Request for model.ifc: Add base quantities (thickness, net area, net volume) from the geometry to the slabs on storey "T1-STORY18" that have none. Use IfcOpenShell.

First a look at what the model holds.

```python
import ifcopenshell
import ifcopenshell.util.element
import ifcopenshell.util.unit

model = ifcopenshell.open("model.ifc")
print(model.schema)
for unit_type in ("LENGTHUNIT", "AREAUNIT", "VOLUMEUNIT"):
    print(unit_type, ifcopenshell.util.unit.calculate_unit_scale(model, unit_type))
storey = next(s for s in model.by_type("IfcBuildingStorey") if s.Name == "T1-STORY18")
slabs = [e for e in ifcopenshell.util.element.get_decomposition(storey) if e.is_a("IfcSlab")]
for e in sorted(slabs, key=lambda e: e.id()):
    print(e.id(), e.is_a(), e.Name, list(ifcopenshell.util.element.get_psets(e, qtos_only=True)), sep=" | ")
```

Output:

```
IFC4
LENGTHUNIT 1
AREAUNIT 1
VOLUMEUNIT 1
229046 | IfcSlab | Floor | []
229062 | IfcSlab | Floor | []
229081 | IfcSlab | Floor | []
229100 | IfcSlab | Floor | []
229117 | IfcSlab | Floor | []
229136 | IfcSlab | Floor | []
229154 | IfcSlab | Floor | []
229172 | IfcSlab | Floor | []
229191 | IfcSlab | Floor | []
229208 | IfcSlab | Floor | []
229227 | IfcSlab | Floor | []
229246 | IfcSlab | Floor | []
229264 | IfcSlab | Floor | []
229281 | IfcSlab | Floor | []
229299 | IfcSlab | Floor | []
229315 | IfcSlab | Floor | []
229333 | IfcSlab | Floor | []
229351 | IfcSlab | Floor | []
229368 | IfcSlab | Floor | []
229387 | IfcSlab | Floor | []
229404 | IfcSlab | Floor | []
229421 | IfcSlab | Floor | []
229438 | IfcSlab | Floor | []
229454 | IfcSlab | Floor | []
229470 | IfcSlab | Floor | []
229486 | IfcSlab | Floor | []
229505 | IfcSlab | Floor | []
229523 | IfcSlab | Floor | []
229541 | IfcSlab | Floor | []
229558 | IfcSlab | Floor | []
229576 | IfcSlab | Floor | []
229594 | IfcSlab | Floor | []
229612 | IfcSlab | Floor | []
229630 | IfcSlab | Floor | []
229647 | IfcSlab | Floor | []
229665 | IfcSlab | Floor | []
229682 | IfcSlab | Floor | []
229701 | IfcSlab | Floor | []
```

```python
import ifcopenshell
import ifcopenshell.api.pset
import ifcopenshell.geom
import ifcopenshell.util.element
import ifcopenshell.util.shape
import ifcopenshell.util.unit

model = ifcopenshell.open("model.ifc")
unit_scale = ifcopenshell.util.unit.calculate_unit_scale(model)
area_scale = ifcopenshell.util.unit.calculate_unit_scale(model, "AREAUNIT")
volume_scale = ifcopenshell.util.unit.calculate_unit_scale(model, "VOLUMEUNIT")
settings = ifcopenshell.geom.settings()

storey = next(s for s in model.by_type("IfcBuildingStorey") if s.Name == "T1-STORY18")
slabs = [e for e in ifcopenshell.util.element.get_decomposition(storey) if e.is_a("IfcSlab")]

for e in sorted(slabs, key=lambda e: e.id()):
    if ifcopenshell.util.element.get_psets(e, qtos_only=True, should_inherit=False):
        continue
    # Geometry comes back in metres, in the element's own axes.
    shape = ifcopenshell.geom.create_shape(settings, e)
    values = {
        "Width": ifcopenshell.util.shape.get_z(shape.geometry) / unit_scale,
        "NetArea": ifcopenshell.util.shape.get_footprint_area(shape.geometry) / area_scale,
        "NetVolume": ifcopenshell.util.shape.get_volume(shape.geometry) / volume_scale,
    }
    qto = ifcopenshell.api.pset.add_qto(model, product=e, name="Qto_SlabBaseQuantities")
    ifcopenshell.api.pset.edit_qto(model, qto=qto, properties=values)
    print(e.id(), {k: round(v, 3) for k, v in values.items()})

model.write("model_updated.ifc")
```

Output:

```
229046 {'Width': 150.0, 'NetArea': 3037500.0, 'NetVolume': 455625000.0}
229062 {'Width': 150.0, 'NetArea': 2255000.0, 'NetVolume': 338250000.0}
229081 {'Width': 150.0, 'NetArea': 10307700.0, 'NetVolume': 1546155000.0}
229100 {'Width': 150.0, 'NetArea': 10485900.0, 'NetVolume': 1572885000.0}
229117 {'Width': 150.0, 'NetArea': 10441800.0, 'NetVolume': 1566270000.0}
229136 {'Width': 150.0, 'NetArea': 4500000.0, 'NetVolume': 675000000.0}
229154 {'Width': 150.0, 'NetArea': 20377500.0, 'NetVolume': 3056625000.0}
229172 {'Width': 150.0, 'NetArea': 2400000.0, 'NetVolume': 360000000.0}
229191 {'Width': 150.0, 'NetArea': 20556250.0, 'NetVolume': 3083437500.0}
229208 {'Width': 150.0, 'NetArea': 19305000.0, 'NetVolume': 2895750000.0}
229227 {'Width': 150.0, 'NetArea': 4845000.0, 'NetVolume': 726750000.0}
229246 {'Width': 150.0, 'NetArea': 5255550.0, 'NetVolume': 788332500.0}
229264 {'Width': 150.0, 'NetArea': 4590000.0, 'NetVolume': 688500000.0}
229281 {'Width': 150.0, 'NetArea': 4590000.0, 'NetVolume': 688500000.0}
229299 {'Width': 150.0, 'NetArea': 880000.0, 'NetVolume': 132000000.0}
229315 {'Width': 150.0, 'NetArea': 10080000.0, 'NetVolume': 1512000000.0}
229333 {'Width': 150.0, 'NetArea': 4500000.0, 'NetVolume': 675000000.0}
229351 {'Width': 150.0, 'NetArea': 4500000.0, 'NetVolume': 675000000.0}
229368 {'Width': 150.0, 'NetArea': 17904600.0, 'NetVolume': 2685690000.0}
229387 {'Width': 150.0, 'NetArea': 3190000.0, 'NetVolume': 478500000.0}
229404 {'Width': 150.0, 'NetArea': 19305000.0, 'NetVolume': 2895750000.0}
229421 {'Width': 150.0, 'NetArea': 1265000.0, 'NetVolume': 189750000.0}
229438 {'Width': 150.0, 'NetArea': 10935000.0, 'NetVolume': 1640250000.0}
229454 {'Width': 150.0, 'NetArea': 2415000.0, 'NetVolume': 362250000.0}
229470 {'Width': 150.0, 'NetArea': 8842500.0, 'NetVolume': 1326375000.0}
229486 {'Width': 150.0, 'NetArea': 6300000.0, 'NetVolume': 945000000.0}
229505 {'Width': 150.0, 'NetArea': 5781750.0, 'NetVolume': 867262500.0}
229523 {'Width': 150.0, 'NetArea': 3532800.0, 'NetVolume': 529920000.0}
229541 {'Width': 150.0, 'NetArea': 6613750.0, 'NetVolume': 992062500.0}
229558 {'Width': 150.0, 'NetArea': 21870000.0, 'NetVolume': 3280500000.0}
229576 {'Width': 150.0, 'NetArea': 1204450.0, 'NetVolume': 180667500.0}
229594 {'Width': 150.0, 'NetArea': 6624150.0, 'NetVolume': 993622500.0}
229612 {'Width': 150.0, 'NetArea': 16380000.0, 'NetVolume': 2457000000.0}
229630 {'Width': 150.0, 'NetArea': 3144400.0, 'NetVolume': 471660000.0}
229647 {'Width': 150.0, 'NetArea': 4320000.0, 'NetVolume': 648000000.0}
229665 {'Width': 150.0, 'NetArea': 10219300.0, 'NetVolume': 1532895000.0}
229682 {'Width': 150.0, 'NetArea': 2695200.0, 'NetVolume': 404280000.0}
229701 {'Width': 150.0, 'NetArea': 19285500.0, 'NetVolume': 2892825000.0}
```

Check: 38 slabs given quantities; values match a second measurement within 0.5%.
